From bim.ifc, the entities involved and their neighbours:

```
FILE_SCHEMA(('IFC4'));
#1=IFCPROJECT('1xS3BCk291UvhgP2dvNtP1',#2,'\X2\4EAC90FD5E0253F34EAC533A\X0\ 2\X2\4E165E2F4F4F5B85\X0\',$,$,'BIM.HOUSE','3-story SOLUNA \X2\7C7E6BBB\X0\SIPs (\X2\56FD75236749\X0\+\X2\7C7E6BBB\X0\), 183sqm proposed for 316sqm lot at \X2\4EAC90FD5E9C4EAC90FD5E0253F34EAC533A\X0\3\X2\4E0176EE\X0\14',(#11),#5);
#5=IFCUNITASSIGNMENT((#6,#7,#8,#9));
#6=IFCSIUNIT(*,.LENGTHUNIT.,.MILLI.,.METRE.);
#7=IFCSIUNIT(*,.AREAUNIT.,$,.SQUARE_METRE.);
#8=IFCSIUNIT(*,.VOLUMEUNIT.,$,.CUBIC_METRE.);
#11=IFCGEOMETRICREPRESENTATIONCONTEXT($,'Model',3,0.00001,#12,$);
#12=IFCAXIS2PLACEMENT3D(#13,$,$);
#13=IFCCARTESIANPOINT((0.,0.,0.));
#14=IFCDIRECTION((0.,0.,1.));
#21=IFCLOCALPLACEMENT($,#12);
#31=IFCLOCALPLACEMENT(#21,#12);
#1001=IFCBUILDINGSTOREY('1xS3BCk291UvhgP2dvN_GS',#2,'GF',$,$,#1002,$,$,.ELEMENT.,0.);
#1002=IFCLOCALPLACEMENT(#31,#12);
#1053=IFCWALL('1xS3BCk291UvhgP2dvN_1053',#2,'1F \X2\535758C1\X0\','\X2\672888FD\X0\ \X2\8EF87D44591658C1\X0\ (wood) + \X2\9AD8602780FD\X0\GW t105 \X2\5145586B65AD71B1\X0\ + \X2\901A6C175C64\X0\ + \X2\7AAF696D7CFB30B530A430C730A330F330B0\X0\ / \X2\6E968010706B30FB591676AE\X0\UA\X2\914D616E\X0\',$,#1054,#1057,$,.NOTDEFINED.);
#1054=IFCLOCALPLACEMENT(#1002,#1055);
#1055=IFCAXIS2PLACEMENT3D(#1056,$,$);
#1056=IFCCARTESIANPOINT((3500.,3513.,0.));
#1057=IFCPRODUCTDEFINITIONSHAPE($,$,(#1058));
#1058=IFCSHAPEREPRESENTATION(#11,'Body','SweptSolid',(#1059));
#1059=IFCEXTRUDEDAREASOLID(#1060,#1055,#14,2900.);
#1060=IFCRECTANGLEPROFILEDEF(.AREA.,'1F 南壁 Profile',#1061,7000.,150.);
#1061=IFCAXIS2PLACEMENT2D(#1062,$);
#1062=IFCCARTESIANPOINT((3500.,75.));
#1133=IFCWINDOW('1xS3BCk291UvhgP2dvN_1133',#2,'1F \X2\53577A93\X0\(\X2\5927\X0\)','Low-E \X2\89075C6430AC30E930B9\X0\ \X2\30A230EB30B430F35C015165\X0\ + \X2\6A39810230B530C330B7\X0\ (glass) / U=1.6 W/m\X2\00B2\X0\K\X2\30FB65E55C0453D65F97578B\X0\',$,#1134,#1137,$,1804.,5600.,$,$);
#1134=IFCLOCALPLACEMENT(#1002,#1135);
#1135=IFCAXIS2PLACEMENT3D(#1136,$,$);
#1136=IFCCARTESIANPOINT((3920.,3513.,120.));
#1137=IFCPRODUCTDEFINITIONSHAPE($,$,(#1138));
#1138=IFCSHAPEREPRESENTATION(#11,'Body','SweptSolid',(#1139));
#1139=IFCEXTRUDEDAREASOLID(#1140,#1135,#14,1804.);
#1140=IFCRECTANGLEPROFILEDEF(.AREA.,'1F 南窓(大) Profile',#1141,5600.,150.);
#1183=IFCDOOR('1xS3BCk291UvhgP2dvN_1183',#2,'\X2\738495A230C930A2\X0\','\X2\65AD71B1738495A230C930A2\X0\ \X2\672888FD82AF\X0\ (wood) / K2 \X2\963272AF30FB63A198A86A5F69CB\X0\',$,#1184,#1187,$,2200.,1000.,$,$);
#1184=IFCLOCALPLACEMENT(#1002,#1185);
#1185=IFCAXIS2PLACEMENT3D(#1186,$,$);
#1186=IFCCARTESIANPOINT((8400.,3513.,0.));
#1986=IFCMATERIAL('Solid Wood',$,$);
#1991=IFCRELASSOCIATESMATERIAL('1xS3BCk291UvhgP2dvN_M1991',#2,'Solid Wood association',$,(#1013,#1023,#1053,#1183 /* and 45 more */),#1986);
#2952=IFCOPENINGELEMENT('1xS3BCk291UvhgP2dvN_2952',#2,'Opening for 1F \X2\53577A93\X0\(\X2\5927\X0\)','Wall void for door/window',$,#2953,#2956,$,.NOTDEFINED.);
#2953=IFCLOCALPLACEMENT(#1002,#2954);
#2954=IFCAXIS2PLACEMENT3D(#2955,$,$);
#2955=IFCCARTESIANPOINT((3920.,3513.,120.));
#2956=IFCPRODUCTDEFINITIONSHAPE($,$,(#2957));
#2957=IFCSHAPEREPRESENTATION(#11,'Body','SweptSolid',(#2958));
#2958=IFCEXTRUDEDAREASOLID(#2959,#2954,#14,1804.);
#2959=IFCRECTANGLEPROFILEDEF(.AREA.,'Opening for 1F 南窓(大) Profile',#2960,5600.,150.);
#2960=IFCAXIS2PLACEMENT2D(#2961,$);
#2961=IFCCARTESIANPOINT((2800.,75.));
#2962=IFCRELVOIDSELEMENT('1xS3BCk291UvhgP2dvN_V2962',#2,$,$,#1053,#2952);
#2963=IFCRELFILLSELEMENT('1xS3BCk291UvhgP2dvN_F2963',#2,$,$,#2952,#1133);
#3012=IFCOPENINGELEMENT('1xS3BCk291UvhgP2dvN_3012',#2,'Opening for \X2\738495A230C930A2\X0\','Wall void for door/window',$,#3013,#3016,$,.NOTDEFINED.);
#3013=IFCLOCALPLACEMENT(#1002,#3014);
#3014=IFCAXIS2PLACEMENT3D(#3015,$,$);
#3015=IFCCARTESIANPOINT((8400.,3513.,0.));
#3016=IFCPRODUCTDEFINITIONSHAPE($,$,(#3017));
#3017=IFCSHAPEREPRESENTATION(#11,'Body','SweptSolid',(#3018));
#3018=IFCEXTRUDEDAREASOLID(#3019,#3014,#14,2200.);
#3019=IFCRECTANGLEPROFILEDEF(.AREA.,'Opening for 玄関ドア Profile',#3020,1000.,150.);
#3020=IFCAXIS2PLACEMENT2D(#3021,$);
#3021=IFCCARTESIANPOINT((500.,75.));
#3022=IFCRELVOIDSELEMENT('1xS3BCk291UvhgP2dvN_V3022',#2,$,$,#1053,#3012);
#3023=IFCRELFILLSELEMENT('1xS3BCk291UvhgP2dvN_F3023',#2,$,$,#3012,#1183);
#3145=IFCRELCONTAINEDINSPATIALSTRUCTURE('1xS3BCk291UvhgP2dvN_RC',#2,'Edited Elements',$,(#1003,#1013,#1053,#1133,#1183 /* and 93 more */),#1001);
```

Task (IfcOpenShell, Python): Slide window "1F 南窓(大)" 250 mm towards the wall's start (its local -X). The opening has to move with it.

```python
import ifcopenshell
import ifcopenshell.api.geometry
import ifcopenshell.util.placement
import ifcopenshell.util.unit

model = ifcopenshell.open("bim.ifc")
unit_scale = ifcopenshell.util.unit.calculate_unit_scale(model)

window = model.by_id(1133)
opening = window.FillsVoids[0].RelatingOpeningElement
wall = opening.VoidsElements[0].RelatingBuildingElement

wall_matrix = ifcopenshell.util.placement.get_local_placement(wall.ObjectPlacement)
shift = wall_matrix[:3, 0] * -0.25 / unit_scale
before = ifcopenshell.util.placement.get_local_placement(window.ObjectPlacement)[:3, 3].copy()

# The window is not placed relative to its opening, so move both.
for product in (opening, window):
    matrix = ifcopenshell.util.placement.get_local_placement(product.ObjectPlacement)
    matrix[:3, 3] += shift
    ifcopenshell.api.geometry.edit_object_placement(model, product=product, matrix=matrix, is_si=False)

after = ifcopenshell.util.placement.get_local_placement(window.ObjectPlacement)[:3, 3]
print("window moved by", (after - before).round(3) + 0.0)

model.write("bim_v2.ifc")
```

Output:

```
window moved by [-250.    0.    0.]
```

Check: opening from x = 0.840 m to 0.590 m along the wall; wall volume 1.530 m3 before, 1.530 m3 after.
